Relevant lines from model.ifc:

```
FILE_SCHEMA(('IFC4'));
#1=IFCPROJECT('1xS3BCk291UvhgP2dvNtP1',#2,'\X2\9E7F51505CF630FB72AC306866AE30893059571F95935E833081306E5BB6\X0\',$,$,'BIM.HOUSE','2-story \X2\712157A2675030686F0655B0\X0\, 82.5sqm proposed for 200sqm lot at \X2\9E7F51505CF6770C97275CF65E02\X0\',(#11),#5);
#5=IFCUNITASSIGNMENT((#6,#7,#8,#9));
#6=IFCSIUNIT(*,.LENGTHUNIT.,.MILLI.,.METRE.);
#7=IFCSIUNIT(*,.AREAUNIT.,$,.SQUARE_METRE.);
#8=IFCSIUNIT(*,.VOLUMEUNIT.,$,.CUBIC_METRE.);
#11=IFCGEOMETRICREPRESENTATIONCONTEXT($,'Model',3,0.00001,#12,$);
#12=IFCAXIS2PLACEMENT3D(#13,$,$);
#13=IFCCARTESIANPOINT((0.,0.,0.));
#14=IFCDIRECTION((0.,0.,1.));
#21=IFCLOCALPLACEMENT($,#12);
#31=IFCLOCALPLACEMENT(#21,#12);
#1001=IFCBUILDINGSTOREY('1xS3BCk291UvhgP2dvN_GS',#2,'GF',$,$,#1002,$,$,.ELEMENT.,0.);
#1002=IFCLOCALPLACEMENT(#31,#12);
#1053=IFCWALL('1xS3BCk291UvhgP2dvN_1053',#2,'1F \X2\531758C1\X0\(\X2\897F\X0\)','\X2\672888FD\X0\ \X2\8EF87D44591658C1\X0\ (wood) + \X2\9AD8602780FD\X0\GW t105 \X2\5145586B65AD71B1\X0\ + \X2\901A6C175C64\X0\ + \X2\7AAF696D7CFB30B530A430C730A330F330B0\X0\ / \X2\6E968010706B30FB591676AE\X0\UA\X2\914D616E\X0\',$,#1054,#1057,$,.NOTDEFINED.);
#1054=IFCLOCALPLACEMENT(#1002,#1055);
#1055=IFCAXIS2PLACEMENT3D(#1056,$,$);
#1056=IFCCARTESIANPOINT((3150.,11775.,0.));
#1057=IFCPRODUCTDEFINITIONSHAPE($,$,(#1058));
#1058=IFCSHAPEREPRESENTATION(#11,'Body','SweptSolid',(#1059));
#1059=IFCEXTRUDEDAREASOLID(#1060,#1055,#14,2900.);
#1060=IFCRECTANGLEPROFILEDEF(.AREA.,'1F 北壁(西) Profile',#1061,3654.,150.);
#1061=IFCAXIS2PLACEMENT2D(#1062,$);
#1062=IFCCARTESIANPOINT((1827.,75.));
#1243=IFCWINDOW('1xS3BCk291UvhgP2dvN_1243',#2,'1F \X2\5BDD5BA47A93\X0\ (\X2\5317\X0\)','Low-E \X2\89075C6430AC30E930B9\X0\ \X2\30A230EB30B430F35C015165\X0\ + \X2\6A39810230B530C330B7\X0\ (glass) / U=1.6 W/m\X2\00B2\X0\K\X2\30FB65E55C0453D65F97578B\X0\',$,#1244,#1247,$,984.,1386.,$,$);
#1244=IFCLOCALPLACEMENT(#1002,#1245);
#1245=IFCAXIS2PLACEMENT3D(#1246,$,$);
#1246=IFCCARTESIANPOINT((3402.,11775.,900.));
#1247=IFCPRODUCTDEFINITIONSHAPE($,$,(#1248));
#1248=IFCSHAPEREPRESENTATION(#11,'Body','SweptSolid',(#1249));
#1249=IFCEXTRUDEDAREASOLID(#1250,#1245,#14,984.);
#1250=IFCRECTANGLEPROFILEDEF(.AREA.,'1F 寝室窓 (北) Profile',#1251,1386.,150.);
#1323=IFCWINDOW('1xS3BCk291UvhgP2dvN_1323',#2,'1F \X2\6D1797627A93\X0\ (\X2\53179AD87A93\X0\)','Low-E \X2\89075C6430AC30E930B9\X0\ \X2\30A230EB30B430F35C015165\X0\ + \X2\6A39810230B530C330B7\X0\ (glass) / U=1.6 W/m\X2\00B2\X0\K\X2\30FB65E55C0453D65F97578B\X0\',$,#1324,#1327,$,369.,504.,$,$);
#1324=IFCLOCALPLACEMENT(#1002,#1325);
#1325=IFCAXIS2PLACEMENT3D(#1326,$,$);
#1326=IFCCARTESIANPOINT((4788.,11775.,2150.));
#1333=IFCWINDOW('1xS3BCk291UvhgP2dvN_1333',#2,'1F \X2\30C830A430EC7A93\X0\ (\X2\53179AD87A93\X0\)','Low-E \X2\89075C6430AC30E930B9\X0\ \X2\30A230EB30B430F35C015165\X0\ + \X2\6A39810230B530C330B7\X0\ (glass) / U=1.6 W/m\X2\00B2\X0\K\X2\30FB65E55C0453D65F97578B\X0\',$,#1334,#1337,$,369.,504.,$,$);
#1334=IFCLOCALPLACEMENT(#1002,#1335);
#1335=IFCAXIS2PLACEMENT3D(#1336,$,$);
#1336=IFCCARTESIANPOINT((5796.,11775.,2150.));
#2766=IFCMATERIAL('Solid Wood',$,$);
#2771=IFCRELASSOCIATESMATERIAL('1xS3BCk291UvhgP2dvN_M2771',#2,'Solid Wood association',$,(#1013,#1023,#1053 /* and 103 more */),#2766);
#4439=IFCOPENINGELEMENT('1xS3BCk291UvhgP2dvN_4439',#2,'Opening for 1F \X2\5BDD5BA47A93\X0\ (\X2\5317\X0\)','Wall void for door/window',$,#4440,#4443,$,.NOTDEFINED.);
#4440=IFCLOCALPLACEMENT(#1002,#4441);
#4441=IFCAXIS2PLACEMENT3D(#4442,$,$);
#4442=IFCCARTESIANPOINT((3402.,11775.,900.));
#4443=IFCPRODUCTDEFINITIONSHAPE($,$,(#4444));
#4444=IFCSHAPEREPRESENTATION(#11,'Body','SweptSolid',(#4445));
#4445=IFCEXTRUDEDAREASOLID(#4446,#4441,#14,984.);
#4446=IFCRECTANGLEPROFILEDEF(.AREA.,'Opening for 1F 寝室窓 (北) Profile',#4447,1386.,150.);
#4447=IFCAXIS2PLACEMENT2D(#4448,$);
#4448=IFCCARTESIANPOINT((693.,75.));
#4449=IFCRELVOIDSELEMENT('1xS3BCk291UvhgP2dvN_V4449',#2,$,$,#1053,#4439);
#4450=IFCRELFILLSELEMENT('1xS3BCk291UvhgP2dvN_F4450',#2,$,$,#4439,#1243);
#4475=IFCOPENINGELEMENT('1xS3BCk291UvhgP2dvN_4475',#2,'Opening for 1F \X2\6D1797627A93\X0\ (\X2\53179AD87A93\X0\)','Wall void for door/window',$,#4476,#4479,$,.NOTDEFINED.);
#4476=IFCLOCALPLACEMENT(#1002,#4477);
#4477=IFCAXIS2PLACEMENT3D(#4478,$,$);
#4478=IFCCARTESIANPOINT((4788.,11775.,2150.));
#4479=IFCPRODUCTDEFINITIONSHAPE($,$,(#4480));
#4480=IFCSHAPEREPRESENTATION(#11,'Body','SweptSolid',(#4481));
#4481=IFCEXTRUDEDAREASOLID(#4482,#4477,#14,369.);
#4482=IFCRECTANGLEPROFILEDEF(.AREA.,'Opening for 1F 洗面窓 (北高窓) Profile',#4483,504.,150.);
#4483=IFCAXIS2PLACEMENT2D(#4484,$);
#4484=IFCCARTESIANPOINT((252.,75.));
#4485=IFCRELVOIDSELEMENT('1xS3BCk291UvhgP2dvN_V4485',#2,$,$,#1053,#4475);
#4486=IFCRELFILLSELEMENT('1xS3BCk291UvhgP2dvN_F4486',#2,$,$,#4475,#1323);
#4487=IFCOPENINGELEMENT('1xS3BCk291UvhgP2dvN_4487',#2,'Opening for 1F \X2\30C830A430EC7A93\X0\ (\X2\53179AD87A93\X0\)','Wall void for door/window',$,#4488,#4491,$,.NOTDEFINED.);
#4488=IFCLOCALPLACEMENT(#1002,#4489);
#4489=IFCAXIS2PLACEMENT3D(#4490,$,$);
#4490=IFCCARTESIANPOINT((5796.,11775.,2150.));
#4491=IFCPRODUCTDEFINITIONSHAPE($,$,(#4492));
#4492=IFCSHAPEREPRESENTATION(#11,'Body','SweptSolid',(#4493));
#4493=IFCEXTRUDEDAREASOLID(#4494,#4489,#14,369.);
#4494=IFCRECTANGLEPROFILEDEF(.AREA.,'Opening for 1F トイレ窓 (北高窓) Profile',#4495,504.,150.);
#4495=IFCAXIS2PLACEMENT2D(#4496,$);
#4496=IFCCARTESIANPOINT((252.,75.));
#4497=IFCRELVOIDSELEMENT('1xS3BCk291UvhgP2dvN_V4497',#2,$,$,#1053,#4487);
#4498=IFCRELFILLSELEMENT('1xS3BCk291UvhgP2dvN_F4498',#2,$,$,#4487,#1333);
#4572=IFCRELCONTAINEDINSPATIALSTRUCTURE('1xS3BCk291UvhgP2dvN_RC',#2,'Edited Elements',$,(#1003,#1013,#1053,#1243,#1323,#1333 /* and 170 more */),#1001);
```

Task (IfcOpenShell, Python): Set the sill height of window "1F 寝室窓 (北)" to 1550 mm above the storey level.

```python
import numpy as np
import ifcopenshell
import ifcopenshell.api.geometry
import ifcopenshell.geom
import ifcopenshell.util.element
import ifcopenshell.util.placement
import ifcopenshell.util.shape
import ifcopenshell.util.unit

model = ifcopenshell.open("model.ifc")
unit_scale = ifcopenshell.util.unit.calculate_unit_scale(model)

window = model.by_id(1243)
opening = window.FillsVoids[0].RelatingOpeningElement
storey = ifcopenshell.util.element.get_container(window, ifc_class="IfcBuildingStorey")
level = ifcopenshell.util.placement.get_local_placement(storey.ObjectPlacement)[2, 3]

# The opening's origin need not be at the sill, so measure its lowest point.
shape = ifcopenshell.geom.create_shape(ifcopenshell.geom.settings(), opening)
bottom = ifcopenshell.util.shape.get_shape_bottom_elevation(shape, shape.geometry) / unit_scale
dz = level + 1550.0 - bottom

shift = np.array([0.0, 0.0, dz])
# The window is not placed relative to its opening, so move both.
for product in (opening, window):
    matrix = ifcopenshell.util.placement.get_local_placement(product.ObjectPlacement)
    matrix[:3, 3] += shift
    ifcopenshell.api.geometry.edit_object_placement(model, product=product, matrix=matrix, is_si=False)

print(f"moved by {dz * unit_scale:+.3f} m")

model.write("model_edited.ifc")
```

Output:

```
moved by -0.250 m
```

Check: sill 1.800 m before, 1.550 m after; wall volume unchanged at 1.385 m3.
